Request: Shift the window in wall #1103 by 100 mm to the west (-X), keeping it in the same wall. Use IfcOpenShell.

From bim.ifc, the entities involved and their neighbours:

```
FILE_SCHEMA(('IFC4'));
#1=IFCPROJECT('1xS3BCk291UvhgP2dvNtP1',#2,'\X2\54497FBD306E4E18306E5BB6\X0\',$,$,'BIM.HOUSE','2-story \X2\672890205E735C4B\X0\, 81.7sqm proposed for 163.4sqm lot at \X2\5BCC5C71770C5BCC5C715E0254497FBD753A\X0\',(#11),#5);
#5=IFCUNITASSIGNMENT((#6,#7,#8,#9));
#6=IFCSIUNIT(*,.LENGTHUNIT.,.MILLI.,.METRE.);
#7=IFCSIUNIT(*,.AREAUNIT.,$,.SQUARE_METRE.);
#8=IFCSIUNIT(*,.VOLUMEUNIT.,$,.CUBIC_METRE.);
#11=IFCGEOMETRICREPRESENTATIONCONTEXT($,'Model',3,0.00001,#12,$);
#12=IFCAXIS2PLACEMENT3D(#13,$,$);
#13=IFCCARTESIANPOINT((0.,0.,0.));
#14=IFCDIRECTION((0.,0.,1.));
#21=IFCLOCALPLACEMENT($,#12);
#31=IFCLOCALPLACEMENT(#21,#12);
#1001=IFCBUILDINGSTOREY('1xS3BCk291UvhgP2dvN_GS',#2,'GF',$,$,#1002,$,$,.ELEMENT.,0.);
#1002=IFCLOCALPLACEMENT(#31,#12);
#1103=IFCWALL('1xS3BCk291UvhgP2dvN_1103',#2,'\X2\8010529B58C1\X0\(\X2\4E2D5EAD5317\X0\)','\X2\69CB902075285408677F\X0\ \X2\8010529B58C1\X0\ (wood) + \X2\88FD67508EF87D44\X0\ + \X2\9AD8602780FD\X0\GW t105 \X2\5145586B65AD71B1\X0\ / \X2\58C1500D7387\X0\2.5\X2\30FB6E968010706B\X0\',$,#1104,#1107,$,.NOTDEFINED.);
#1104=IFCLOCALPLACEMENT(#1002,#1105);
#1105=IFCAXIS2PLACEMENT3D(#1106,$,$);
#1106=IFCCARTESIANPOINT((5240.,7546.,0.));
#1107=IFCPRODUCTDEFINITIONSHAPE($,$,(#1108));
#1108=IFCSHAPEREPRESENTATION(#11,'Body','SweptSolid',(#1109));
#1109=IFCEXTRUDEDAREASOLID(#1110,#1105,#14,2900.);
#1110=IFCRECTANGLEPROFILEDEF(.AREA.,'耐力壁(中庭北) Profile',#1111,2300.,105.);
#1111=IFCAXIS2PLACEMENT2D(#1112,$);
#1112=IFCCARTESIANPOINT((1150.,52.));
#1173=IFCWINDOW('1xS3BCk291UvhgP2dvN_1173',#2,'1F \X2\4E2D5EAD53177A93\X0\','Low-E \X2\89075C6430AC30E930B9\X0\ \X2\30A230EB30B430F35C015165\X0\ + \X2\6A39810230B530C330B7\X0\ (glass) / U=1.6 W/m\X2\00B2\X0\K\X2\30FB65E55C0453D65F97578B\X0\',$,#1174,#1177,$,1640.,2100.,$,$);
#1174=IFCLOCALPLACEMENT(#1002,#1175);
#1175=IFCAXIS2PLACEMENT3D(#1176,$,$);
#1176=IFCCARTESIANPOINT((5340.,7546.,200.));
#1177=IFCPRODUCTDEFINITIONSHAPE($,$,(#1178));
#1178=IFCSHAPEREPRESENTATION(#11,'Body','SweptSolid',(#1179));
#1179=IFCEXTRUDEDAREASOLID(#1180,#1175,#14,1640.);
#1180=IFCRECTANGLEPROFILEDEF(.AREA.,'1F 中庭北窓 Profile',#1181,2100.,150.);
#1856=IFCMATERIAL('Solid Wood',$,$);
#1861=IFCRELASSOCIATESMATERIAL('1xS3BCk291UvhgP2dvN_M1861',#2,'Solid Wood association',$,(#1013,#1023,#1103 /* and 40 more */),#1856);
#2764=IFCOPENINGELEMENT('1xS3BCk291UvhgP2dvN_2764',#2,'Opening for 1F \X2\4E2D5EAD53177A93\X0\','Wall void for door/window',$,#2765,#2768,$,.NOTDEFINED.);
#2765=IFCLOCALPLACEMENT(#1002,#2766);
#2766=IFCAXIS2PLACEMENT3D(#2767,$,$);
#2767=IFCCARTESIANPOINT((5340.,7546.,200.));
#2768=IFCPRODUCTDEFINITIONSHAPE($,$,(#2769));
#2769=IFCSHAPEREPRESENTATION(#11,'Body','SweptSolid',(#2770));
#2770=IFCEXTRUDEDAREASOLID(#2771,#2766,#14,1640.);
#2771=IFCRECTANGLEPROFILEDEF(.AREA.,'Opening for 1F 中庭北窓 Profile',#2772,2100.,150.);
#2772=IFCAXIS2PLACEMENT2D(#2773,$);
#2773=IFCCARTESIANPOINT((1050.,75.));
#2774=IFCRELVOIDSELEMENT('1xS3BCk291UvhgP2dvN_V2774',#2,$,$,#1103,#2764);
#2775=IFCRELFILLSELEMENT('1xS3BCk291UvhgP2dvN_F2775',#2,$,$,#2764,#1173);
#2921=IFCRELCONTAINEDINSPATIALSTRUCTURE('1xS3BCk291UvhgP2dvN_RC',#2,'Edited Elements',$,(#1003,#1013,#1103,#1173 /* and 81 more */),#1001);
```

```python
import ifcopenshell
import ifcopenshell.api.geometry
import ifcopenshell.util.placement

model = ifcopenshell.open("bim.ifc")

window = model.by_id(1173)
opening = window.FillsVoids[0].RelatingOpeningElement
wall = opening.VoidsElements[0].RelatingBuildingElement

wall_matrix = ifcopenshell.util.placement.get_local_placement(wall.ObjectPlacement)
shift = wall_matrix[:3, 0] * -100.0
before = ifcopenshell.util.placement.get_local_placement(window.ObjectPlacement)[:3, 3].copy()

# The window is not placed relative to its opening, so move both.
for product in (opening, window):
    matrix = ifcopenshell.util.placement.get_local_placement(product.ObjectPlacement)
    matrix[:3, 3] += shift
    ifcopenshell.api.geometry.edit_object_placement(model, product=product, matrix=matrix, is_si=False)

after = ifcopenshell.util.placement.get_local_placement(window.ObjectPlacement)[:3, 3]
print("window moved by", (after - before).round(3) + 0.0)

model.write("bim_edited.ifc")
```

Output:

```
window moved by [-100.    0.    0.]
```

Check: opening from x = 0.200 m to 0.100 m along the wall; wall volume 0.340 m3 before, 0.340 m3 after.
